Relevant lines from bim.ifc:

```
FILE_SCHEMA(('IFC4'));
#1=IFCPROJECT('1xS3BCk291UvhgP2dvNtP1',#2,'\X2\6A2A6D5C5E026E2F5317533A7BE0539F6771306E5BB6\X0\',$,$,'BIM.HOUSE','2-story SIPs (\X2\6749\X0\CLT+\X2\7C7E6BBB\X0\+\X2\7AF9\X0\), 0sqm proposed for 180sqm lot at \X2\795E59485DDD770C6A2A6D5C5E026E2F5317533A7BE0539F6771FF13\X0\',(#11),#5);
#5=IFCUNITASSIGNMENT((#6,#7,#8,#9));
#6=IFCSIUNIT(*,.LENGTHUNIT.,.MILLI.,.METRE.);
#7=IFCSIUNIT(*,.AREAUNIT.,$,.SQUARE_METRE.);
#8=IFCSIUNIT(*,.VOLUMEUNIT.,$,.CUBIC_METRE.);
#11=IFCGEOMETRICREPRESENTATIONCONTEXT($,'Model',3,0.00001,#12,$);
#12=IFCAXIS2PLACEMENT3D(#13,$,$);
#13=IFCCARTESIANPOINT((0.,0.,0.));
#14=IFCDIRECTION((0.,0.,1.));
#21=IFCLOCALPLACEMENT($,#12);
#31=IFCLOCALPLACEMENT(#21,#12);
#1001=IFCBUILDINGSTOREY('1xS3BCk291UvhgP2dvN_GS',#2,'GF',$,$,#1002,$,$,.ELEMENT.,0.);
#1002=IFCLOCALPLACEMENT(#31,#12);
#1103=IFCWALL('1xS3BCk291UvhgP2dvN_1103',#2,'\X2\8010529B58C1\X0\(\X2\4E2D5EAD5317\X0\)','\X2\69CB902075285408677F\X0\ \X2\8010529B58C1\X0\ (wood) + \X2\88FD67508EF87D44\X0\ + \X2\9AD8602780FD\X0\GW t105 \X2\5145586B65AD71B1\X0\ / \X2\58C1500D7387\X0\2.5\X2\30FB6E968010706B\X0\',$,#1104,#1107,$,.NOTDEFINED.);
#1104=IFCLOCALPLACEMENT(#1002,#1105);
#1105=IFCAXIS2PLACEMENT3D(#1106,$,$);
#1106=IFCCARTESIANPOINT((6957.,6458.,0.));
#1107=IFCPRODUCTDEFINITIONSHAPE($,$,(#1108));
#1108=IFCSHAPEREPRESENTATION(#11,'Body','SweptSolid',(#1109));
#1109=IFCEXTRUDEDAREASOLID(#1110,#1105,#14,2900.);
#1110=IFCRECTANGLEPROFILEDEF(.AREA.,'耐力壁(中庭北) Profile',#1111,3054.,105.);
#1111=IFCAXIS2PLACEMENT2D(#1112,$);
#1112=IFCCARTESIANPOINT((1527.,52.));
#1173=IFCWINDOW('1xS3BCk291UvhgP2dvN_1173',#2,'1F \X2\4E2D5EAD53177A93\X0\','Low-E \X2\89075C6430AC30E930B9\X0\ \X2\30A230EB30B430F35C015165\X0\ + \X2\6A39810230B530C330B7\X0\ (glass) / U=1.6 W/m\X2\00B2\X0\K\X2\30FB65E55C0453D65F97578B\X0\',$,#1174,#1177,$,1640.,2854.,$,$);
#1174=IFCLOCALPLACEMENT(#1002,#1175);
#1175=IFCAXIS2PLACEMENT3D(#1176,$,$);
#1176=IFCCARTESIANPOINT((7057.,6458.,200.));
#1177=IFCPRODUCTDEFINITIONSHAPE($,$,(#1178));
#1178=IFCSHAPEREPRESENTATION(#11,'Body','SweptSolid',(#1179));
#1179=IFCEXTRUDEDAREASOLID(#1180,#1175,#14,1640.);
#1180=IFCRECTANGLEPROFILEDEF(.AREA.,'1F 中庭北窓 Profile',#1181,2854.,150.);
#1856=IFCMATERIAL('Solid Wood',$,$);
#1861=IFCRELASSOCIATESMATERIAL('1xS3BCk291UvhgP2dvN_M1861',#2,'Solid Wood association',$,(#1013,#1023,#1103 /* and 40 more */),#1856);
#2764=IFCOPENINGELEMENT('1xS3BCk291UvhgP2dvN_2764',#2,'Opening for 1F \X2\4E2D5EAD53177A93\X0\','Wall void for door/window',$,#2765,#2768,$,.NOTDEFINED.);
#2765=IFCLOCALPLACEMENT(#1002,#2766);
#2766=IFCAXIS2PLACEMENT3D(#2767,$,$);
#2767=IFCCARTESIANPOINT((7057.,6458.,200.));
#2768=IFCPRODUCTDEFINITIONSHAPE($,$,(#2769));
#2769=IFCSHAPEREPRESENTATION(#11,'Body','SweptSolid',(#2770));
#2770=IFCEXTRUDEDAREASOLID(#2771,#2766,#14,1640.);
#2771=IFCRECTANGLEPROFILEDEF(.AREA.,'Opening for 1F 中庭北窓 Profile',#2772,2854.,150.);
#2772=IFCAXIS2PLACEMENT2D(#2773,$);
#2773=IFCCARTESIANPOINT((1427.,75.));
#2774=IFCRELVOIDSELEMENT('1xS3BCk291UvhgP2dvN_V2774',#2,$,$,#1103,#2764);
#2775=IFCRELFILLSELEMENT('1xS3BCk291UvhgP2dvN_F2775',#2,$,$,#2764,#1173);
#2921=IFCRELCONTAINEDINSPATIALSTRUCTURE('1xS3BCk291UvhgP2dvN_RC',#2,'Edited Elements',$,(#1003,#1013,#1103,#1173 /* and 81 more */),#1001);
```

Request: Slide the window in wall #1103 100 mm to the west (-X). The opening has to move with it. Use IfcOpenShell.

```python
import ifcopenshell
import ifcopenshell.api.geometry
import ifcopenshell.util.placement
import ifcopenshell.util.unit

model = ifcopenshell.open("bim.ifc")
unit_scale = ifcopenshell.util.unit.calculate_unit_scale(model)

window = model.by_guid("1xS3BCk291UvhgP2dvN_1173")
opening = window.FillsVoids[0].RelatingOpeningElement
wall = opening.VoidsElements[0].RelatingBuildingElement

wall_matrix = ifcopenshell.util.placement.get_local_placement(wall.ObjectPlacement)
shift = wall_matrix[:3, 0] * -0.1 / unit_scale
before = ifcopenshell.util.placement.get_local_placement(window.ObjectPlacement)[:3, 3].copy()

# The window is not placed relative to its opening, so move both.
for product in (opening, window):
    matrix = ifcopenshell.util.placement.get_local_placement(product.ObjectPlacement)
    matrix[:3, 3] += shift
    ifcopenshell.api.geometry.edit_object_placement(model, product=product, matrix=matrix, is_si=False)

after = ifcopenshell.util.placement.get_local_placement(window.ObjectPlacement)[:3, 3]
print("window moved by", (after - before).round(3) + 0.0)

model.write("bim_rev.ifc")
```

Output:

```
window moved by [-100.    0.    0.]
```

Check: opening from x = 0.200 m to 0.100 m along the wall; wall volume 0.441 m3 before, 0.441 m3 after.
